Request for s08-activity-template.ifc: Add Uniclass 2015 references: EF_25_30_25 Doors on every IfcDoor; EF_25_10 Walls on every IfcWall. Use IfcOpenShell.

First a look at what the model holds.

```python
import ifcopenshell

model = ifcopenshell.open("s08-activity-template.ifc")
print(model.schema)
print("classifications:", [c.Name for c in model.by_type("IfcClassification")])
for ifc_class in ("IfcDoor", "IfcRoof", "IfcStair", "IfcWall", "IfcWindow"):
    print(ifc_class, len(model.by_type(ifc_class)))
```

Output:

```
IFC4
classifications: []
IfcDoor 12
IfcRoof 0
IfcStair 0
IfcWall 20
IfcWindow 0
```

```python
import ifcopenshell
import ifcopenshell.api.classification

model = ifcopenshell.open("s08-activity-template.ifc")

system = ifcopenshell.api.classification.add_classification(model, classification="Uniclass 2015")

codes = {
    "IfcDoor": ("EF_25_30_25", "Doors"),
    "IfcWall": ("EF_25_10", "Walls"),
}
for ifc_class, (code, name) in codes.items():
    products = model.by_type(ifc_class)
    ifcopenshell.api.classification.add_reference(
        model, products=products, classification=system, identification=code, name=name
    )
    print(code, len(products))

model.write("s08-activity-template_updated.ifc")
```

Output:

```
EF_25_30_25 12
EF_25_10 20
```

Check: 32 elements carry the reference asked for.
